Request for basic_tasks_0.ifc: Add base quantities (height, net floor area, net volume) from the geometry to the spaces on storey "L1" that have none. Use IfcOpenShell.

First a look at what the model holds.

```python
import ifcopenshell
import ifcopenshell.util.element
import ifcopenshell.util.unit

model = ifcopenshell.open("basic_tasks_0.ifc")
print(model.schema)
for unit_type in ("LENGTHUNIT", "AREAUNIT", "VOLUMEUNIT"):
    print(unit_type, ifcopenshell.util.unit.calculate_unit_scale(model, unit_type))
storey = next(s for s in model.by_type("IfcBuildingStorey") if s.Name == "L1")
spaces = [e for e in ifcopenshell.util.element.get_decomposition(storey) if e.is_a("IfcSpace")]
for e in sorted(spaces, key=lambda e: e.id()):
    print(e.id(), e.is_a(), e.Name, list(ifcopenshell.util.element.get_psets(e, qtos_only=True)), sep=" | ")
```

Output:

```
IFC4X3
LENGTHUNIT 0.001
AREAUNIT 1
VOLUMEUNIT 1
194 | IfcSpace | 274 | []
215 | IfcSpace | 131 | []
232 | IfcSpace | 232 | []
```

```python
import ifcopenshell
import ifcopenshell.api.pset
import ifcopenshell.geom
import ifcopenshell.util.element
import ifcopenshell.util.shape
import ifcopenshell.util.unit

model = ifcopenshell.open("basic_tasks_0.ifc")
unit_scale = ifcopenshell.util.unit.calculate_unit_scale(model)
area_scale = ifcopenshell.util.unit.calculate_unit_scale(model, "AREAUNIT")
volume_scale = ifcopenshell.util.unit.calculate_unit_scale(model, "VOLUMEUNIT")
settings = ifcopenshell.geom.settings()

storey = next(s for s in model.by_type("IfcBuildingStorey") if s.Name == "L1")
spaces = [e for e in ifcopenshell.util.element.get_decomposition(storey) if e.is_a("IfcSpace")]

for e in sorted(spaces, key=lambda e: e.id()):
    if ifcopenshell.util.element.get_psets(e, qtos_only=True, should_inherit=False):
        continue
    # Geometry comes back in metres, in the element's own axes.
    shape = ifcopenshell.geom.create_shape(settings, e)
    values = {
        "Height": ifcopenshell.util.shape.get_z(shape.geometry) / unit_scale,
        "NetFloorArea": ifcopenshell.util.shape.get_footprint_area(shape.geometry) / area_scale,
        "NetVolume": ifcopenshell.util.shape.get_volume(shape.geometry) / volume_scale,
    }
    qto = ifcopenshell.api.pset.add_qto(model, product=e, name="Qto_SpaceBaseQuantities")
    ifcopenshell.api.pset.edit_qto(model, qto=qto, properties=values)
    print(e.id(), {k: round(v, 3) for k, v in values.items()})

model.write("basic_tasks_0-out.ifc")
```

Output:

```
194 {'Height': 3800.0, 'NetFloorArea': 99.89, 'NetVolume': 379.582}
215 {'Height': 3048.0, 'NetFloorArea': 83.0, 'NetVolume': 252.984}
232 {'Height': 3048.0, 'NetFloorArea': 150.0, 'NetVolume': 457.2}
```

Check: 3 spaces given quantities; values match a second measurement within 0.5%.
